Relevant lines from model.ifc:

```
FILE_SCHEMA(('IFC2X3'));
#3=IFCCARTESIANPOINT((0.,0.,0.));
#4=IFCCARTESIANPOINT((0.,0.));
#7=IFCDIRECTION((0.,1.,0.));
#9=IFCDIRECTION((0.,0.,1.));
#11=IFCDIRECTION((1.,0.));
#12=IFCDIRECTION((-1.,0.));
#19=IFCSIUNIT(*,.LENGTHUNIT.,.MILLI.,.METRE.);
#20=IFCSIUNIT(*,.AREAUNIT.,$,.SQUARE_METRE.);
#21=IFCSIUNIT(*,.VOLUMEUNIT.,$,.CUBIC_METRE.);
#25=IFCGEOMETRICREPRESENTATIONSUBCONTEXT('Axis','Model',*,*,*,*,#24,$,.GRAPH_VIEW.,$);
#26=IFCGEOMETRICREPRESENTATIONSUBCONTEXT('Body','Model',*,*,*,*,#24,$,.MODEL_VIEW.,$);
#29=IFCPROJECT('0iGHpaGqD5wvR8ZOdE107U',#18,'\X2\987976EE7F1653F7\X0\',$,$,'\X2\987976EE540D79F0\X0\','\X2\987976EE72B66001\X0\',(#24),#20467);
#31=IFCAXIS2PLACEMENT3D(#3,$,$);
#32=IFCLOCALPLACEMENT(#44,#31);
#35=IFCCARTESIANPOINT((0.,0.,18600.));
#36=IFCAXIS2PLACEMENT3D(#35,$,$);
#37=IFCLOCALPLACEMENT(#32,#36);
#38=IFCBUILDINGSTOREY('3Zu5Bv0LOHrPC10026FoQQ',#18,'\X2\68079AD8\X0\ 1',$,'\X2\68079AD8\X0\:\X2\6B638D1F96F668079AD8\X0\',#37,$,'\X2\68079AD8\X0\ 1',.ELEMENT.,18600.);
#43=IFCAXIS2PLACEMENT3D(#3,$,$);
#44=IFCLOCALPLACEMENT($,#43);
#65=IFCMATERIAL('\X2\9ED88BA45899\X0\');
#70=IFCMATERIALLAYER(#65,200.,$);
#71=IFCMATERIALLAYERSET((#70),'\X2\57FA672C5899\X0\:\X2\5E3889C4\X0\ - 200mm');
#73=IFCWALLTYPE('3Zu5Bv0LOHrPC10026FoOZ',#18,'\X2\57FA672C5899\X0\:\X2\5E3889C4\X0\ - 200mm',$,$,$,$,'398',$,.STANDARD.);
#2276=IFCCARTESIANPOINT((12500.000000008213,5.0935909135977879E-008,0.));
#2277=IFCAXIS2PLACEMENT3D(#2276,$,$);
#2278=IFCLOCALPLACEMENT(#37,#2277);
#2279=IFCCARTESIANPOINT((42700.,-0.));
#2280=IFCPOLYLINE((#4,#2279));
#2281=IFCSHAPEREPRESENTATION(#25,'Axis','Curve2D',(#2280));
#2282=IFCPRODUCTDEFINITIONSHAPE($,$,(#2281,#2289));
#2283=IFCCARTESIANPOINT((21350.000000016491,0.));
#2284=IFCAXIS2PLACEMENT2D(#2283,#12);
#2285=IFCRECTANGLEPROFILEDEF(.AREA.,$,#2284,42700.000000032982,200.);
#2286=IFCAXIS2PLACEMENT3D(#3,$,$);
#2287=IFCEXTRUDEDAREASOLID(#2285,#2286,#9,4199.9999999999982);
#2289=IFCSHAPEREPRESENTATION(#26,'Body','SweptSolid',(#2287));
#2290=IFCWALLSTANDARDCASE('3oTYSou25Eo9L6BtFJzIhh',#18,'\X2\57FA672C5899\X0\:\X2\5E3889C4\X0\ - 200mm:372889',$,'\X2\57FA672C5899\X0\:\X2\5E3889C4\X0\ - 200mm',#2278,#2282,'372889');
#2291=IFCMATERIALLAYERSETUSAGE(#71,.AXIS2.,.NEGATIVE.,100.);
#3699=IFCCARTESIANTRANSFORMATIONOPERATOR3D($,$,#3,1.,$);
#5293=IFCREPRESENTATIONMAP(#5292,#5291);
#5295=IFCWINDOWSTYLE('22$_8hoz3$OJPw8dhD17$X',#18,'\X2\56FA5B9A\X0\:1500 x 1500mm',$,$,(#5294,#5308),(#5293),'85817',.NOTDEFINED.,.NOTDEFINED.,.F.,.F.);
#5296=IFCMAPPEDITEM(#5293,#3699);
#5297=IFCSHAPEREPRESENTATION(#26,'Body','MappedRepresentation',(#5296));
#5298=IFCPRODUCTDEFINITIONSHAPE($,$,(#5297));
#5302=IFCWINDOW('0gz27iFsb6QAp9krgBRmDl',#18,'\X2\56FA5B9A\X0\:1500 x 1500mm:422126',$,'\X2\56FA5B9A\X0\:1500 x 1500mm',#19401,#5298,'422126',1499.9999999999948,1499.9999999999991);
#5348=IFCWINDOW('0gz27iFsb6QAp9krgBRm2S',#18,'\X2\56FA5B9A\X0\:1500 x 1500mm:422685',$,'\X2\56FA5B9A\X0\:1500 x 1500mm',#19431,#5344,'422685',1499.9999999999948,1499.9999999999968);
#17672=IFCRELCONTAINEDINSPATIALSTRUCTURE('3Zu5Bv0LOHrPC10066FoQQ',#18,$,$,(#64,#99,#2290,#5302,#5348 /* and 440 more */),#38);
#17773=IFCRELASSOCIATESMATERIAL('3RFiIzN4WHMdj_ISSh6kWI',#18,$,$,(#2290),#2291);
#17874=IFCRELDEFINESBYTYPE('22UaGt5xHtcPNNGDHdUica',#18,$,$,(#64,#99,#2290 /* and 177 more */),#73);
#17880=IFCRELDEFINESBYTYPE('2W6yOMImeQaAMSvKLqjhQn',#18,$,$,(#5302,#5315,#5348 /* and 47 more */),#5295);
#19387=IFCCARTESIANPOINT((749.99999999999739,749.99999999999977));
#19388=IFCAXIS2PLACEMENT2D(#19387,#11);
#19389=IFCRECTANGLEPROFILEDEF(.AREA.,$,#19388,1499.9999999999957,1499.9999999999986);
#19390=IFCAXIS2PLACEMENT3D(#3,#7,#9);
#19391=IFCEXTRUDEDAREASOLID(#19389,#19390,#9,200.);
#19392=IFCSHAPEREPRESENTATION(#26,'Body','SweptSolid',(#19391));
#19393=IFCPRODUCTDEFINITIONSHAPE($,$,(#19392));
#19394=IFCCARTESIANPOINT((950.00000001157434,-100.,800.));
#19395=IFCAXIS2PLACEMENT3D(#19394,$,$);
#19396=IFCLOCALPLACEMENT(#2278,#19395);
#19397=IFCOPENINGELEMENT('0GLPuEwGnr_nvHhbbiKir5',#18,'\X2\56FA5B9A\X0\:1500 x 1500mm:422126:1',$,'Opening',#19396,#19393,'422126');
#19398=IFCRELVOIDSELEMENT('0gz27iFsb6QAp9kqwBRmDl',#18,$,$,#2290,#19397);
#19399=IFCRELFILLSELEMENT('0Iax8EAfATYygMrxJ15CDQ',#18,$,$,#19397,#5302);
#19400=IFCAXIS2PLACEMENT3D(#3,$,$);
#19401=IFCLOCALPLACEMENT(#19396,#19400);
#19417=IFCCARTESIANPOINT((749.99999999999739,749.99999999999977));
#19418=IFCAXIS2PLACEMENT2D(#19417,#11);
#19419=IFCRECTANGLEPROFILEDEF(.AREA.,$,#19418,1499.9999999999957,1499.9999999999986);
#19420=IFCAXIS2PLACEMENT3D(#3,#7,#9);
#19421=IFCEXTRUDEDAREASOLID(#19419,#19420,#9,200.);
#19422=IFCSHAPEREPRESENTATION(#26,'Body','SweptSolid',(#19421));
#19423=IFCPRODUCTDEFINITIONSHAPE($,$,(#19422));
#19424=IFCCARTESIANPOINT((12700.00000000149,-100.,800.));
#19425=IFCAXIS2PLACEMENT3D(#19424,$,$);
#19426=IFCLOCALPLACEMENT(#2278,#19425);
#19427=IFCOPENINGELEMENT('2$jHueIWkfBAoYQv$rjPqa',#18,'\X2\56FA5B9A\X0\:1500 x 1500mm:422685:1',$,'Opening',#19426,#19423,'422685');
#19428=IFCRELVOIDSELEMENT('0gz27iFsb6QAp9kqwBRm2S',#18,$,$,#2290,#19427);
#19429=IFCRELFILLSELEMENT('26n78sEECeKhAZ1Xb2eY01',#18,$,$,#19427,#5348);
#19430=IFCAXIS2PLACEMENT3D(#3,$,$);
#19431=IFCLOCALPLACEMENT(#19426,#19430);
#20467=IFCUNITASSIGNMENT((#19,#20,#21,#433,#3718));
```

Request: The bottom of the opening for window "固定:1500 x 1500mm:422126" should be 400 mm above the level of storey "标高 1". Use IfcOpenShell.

```python
import numpy as np
import ifcopenshell
import ifcopenshell.api.geometry
import ifcopenshell.geom
import ifcopenshell.util.element
import ifcopenshell.util.placement
import ifcopenshell.util.shape
import ifcopenshell.util.unit

model = ifcopenshell.open("model.ifc")
unit_scale = ifcopenshell.util.unit.calculate_unit_scale(model)

window = model.by_guid("0gz27iFsb6QAp9krgBRmDl")
opening = window.FillsVoids[0].RelatingOpeningElement
storey = ifcopenshell.util.element.get_container(window, ifc_class="IfcBuildingStorey")
level = ifcopenshell.util.placement.get_local_placement(storey.ObjectPlacement)[2, 3]

# The opening's origin need not be at the sill, so measure its lowest point.
shape = ifcopenshell.geom.create_shape(ifcopenshell.geom.settings(), opening)
bottom = ifcopenshell.util.shape.get_shape_bottom_elevation(shape, shape.geometry) / unit_scale
dz = level + 0.4 / unit_scale - bottom

shift = np.array([0.0, 0.0, dz])
# The window is placed relative to its opening, so it follows when the opening moves.
matrix = ifcopenshell.util.placement.get_local_placement(opening.ObjectPlacement)
matrix[:3, 3] += shift
ifcopenshell.api.geometry.edit_object_placement(
    model, product=opening, matrix=matrix, is_si=False, should_transform_children=True
)

print(f"moved by {dz * unit_scale:+.3f} m")

model.write("model_edited.ifc")
```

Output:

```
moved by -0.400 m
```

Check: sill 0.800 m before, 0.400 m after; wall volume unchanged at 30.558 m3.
